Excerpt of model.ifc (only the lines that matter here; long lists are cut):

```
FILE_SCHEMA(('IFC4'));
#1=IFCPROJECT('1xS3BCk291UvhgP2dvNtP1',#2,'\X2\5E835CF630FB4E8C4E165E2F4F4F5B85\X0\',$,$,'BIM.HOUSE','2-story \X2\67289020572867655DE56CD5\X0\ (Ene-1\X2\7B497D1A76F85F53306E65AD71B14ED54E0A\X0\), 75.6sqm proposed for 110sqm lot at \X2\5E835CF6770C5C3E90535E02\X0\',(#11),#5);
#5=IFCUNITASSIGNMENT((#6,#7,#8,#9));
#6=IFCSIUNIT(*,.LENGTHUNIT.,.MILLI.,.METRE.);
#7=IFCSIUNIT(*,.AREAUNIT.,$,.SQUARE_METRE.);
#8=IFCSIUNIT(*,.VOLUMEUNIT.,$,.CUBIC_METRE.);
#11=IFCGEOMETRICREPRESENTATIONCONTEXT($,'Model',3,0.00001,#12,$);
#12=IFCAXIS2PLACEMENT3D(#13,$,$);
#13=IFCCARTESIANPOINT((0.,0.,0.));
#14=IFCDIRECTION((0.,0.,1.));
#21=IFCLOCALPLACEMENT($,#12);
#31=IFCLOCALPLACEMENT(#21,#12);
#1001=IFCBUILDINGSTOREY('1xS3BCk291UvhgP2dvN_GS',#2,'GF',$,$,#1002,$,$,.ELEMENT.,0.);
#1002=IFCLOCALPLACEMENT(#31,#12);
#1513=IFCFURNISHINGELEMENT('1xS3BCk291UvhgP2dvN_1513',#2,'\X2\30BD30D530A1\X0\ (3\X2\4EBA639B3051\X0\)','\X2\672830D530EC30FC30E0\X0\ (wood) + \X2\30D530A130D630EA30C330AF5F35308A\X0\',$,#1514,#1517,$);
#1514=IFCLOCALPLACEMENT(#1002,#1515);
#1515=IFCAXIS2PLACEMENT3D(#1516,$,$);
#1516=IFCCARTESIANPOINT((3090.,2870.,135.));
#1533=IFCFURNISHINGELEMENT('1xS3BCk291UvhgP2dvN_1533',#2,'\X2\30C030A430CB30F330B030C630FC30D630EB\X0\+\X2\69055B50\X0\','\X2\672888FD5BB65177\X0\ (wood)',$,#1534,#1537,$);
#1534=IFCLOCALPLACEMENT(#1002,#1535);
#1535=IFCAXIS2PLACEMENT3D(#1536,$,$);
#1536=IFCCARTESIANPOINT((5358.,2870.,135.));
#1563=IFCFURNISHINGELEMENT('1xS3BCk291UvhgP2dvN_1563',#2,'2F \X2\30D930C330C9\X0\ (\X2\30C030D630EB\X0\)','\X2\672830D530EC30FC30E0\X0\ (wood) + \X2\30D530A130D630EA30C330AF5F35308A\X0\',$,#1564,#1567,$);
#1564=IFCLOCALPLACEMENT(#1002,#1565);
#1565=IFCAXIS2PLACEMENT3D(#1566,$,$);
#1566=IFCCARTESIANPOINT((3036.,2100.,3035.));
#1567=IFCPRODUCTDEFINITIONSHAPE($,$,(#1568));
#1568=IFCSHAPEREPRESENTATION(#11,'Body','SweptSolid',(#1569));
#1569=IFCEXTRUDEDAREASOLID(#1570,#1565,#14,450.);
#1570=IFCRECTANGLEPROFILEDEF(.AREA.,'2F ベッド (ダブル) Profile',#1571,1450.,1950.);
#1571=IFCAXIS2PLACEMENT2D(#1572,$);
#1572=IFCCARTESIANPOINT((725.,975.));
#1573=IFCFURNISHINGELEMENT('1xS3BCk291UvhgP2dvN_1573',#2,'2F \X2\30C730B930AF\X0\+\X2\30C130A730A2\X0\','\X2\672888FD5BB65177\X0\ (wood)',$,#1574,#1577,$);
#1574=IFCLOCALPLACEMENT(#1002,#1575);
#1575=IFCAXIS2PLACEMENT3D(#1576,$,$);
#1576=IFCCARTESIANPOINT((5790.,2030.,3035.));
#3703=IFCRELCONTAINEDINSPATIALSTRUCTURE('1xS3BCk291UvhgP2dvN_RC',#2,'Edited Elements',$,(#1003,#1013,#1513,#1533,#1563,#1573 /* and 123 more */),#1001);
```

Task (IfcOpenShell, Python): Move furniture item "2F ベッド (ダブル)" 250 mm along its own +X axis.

```python
import ifcopenshell
import ifcopenshell.api.geometry
import ifcopenshell.util.placement
import ifcopenshell.util.unit

model = ifcopenshell.open("model.ifc")
unit_scale = ifcopenshell.util.unit.calculate_unit_scale(model)

item = model.by_id(1563)
matrix = ifcopenshell.util.placement.get_local_placement(item.ObjectPlacement)
matrix[:3, 3] += matrix[:3, 0] * 0.25 / unit_scale
ifcopenshell.api.geometry.edit_object_placement(model, product=item, matrix=matrix, is_si=False)

print(ifcopenshell.util.placement.get_local_placement(item.ObjectPlacement).round(3) + 0.0)

model.write("model_updated.ifc")
```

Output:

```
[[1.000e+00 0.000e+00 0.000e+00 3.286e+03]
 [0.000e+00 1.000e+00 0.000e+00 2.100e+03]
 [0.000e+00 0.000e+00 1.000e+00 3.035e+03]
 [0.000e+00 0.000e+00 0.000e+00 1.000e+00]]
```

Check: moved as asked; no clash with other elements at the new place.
